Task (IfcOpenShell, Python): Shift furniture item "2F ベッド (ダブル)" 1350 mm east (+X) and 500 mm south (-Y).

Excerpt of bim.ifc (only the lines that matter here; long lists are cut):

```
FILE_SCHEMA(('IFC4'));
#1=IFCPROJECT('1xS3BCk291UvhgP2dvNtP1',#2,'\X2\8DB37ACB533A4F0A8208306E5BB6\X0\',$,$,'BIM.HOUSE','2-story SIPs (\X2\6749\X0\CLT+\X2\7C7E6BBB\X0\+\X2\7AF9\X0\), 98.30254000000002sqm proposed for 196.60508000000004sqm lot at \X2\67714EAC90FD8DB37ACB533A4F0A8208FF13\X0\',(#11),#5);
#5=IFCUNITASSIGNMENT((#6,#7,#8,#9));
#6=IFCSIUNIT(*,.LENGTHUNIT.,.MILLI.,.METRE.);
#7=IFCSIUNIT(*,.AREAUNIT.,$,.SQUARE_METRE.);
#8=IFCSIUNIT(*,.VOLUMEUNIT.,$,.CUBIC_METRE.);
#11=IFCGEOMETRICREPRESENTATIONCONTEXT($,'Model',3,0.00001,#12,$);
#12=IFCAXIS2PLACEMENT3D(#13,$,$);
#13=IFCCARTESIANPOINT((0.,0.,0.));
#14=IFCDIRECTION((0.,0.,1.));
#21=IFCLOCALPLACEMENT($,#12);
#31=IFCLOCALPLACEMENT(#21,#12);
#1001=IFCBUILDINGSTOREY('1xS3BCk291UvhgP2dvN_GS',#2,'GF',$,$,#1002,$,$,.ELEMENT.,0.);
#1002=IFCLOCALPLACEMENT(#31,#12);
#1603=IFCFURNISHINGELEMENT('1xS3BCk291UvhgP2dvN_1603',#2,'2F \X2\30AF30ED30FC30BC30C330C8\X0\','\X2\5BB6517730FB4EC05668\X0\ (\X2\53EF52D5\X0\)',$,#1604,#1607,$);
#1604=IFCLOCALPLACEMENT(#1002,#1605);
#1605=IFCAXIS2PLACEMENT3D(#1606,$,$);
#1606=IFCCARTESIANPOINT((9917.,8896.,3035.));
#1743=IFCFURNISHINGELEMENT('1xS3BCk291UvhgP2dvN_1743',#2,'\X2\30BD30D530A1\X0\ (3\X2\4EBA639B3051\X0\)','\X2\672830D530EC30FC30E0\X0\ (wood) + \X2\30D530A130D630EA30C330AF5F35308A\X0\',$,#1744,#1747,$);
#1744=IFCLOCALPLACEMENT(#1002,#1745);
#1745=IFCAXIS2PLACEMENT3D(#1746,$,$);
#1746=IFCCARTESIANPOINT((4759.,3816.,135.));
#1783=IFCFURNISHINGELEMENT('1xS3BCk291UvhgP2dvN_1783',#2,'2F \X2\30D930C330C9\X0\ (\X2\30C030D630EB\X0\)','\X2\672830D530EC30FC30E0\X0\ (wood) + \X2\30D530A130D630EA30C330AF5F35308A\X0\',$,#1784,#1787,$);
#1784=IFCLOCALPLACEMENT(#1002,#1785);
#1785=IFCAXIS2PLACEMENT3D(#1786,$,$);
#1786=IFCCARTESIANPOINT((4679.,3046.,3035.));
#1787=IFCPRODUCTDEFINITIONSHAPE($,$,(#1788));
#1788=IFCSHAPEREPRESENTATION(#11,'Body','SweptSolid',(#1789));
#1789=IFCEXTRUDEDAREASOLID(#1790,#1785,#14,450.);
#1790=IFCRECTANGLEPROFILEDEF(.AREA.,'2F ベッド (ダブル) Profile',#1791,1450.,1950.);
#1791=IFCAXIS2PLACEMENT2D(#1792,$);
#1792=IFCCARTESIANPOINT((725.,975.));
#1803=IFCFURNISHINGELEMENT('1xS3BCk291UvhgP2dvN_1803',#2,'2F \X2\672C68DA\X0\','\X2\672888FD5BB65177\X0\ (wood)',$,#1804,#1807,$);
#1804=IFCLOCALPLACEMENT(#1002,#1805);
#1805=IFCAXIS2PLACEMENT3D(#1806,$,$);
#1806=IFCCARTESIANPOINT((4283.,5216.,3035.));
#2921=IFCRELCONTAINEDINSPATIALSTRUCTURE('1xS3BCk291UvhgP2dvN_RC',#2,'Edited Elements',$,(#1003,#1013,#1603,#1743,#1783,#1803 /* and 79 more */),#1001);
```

```python
import ifcopenshell
import ifcopenshell.api.geometry
import ifcopenshell.util.placement

model = ifcopenshell.open("bim.ifc")

item = model.by_guid("1xS3BCk291UvhgP2dvN_1783")
matrix = ifcopenshell.util.placement.get_local_placement(item.ObjectPlacement)
matrix[0, 3] += 1350.0
matrix[1, 3] -= 500.0
ifcopenshell.api.geometry.edit_object_placement(model, product=item, matrix=matrix, is_si=False)

print(ifcopenshell.util.placement.get_local_placement(item.ObjectPlacement).round(3) + 0.0)

model.write("bim_rev.ifc")
```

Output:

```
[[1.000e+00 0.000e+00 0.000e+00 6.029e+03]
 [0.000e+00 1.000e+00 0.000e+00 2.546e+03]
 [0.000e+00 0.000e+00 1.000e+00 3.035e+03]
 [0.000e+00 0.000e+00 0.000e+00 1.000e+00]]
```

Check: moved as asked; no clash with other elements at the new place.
